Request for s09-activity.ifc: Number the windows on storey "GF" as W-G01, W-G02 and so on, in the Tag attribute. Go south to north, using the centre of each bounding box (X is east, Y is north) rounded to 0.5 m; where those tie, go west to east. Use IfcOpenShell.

First a look at what the model holds.

```python
import ifcopenshell
import ifcopenshell.util.element
import ifcopenshell.util.placement

model = ifcopenshell.open("s09-activity.ifc")
print(model.schema)
storey = next(s for s in model.by_type("IfcBuildingStorey") if s.Name == "GF")
windows = [e for e in ifcopenshell.util.element.get_decomposition(storey) if e.is_a("IfcWindow")]
for e in sorted(windows, key=lambda e: e.id()):
    origin = ifcopenshell.util.placement.get_local_placement(e.ObjectPlacement)[:3, 3]
    print(e.id(), e.Tag, e.Name, origin.round(2) + 0.0, sep=" | ")
```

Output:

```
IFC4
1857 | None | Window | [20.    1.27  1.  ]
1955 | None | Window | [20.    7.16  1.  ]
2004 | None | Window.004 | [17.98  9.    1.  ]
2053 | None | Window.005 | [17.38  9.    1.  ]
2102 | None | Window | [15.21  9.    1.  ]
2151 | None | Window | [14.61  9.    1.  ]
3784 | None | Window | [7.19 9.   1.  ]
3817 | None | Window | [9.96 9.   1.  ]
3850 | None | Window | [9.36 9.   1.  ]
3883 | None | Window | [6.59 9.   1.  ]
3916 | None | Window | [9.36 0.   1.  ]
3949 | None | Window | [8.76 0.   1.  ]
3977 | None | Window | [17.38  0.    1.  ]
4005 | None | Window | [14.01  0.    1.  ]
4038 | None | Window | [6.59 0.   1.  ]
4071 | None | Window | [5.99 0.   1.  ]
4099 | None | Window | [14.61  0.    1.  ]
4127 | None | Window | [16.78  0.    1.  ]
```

```python
import ifcopenshell
import ifcopenshell.geom
import ifcopenshell.util.element
import ifcopenshell.util.shape

model = ifcopenshell.open("s09-activity.ifc")
settings = ifcopenshell.geom.settings()
settings.set("use-world-coords", True)


def centre(element):
    shape = ifcopenshell.geom.create_shape(settings, element)
    return ifcopenshell.util.shape.get_bbox_centroid(shape.geometry)


storey = next(s for s in model.by_type("IfcBuildingStorey") if s.Name == "GF")
windows = [e for e in ifcopenshell.util.element.get_decomposition(storey) if e.is_a("IfcWindow")]

# Insertion points can sit at a corner or the storey origin, so sort by the geometry (in metres).
centres = {e: centre(e) for e in windows}
windows.sort(key=lambda e: (round(centres[e][1] / 0.5), centres[e][0]))

for i, e in enumerate(windows, start=1):
    number = f"W-G{i:02d}"
    e.Tag = number
    print(e.id(), number)

model.write("s09-activity-out.ifc")
```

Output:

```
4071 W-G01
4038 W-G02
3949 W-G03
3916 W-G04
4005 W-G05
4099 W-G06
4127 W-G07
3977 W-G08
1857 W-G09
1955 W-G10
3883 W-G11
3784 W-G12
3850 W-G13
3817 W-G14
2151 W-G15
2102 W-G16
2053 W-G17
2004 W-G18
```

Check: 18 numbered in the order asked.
